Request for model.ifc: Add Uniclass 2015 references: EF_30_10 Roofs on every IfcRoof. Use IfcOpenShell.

First a look at what the model holds.

```python
import ifcopenshell

model = ifcopenshell.open("model.ifc")
print(model.schema)
print("classifications:", [c.Name for c in model.by_type("IfcClassification")])
for ifc_class in ("IfcDoor", "IfcRoof", "IfcStair", "IfcWall", "IfcWindow"):
    print(ifc_class, len(model.by_type(ifc_class)))
```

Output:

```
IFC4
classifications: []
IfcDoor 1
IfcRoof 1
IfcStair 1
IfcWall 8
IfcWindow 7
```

```python
import ifcopenshell
import ifcopenshell.api.classification

model = ifcopenshell.open("model.ifc")

system = ifcopenshell.api.classification.add_classification(model, classification="Uniclass 2015")

codes = {
    "IfcRoof": ("EF_30_10", "Roofs"),
}
for ifc_class, (code, name) in codes.items():
    products = model.by_type(ifc_class)
    ifcopenshell.api.classification.add_reference(
        model, products=products, classification=system, identification=code, name=name
    )
    print(code, len(products))

model.write("model_rev.ifc")
```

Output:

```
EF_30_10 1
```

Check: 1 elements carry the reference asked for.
